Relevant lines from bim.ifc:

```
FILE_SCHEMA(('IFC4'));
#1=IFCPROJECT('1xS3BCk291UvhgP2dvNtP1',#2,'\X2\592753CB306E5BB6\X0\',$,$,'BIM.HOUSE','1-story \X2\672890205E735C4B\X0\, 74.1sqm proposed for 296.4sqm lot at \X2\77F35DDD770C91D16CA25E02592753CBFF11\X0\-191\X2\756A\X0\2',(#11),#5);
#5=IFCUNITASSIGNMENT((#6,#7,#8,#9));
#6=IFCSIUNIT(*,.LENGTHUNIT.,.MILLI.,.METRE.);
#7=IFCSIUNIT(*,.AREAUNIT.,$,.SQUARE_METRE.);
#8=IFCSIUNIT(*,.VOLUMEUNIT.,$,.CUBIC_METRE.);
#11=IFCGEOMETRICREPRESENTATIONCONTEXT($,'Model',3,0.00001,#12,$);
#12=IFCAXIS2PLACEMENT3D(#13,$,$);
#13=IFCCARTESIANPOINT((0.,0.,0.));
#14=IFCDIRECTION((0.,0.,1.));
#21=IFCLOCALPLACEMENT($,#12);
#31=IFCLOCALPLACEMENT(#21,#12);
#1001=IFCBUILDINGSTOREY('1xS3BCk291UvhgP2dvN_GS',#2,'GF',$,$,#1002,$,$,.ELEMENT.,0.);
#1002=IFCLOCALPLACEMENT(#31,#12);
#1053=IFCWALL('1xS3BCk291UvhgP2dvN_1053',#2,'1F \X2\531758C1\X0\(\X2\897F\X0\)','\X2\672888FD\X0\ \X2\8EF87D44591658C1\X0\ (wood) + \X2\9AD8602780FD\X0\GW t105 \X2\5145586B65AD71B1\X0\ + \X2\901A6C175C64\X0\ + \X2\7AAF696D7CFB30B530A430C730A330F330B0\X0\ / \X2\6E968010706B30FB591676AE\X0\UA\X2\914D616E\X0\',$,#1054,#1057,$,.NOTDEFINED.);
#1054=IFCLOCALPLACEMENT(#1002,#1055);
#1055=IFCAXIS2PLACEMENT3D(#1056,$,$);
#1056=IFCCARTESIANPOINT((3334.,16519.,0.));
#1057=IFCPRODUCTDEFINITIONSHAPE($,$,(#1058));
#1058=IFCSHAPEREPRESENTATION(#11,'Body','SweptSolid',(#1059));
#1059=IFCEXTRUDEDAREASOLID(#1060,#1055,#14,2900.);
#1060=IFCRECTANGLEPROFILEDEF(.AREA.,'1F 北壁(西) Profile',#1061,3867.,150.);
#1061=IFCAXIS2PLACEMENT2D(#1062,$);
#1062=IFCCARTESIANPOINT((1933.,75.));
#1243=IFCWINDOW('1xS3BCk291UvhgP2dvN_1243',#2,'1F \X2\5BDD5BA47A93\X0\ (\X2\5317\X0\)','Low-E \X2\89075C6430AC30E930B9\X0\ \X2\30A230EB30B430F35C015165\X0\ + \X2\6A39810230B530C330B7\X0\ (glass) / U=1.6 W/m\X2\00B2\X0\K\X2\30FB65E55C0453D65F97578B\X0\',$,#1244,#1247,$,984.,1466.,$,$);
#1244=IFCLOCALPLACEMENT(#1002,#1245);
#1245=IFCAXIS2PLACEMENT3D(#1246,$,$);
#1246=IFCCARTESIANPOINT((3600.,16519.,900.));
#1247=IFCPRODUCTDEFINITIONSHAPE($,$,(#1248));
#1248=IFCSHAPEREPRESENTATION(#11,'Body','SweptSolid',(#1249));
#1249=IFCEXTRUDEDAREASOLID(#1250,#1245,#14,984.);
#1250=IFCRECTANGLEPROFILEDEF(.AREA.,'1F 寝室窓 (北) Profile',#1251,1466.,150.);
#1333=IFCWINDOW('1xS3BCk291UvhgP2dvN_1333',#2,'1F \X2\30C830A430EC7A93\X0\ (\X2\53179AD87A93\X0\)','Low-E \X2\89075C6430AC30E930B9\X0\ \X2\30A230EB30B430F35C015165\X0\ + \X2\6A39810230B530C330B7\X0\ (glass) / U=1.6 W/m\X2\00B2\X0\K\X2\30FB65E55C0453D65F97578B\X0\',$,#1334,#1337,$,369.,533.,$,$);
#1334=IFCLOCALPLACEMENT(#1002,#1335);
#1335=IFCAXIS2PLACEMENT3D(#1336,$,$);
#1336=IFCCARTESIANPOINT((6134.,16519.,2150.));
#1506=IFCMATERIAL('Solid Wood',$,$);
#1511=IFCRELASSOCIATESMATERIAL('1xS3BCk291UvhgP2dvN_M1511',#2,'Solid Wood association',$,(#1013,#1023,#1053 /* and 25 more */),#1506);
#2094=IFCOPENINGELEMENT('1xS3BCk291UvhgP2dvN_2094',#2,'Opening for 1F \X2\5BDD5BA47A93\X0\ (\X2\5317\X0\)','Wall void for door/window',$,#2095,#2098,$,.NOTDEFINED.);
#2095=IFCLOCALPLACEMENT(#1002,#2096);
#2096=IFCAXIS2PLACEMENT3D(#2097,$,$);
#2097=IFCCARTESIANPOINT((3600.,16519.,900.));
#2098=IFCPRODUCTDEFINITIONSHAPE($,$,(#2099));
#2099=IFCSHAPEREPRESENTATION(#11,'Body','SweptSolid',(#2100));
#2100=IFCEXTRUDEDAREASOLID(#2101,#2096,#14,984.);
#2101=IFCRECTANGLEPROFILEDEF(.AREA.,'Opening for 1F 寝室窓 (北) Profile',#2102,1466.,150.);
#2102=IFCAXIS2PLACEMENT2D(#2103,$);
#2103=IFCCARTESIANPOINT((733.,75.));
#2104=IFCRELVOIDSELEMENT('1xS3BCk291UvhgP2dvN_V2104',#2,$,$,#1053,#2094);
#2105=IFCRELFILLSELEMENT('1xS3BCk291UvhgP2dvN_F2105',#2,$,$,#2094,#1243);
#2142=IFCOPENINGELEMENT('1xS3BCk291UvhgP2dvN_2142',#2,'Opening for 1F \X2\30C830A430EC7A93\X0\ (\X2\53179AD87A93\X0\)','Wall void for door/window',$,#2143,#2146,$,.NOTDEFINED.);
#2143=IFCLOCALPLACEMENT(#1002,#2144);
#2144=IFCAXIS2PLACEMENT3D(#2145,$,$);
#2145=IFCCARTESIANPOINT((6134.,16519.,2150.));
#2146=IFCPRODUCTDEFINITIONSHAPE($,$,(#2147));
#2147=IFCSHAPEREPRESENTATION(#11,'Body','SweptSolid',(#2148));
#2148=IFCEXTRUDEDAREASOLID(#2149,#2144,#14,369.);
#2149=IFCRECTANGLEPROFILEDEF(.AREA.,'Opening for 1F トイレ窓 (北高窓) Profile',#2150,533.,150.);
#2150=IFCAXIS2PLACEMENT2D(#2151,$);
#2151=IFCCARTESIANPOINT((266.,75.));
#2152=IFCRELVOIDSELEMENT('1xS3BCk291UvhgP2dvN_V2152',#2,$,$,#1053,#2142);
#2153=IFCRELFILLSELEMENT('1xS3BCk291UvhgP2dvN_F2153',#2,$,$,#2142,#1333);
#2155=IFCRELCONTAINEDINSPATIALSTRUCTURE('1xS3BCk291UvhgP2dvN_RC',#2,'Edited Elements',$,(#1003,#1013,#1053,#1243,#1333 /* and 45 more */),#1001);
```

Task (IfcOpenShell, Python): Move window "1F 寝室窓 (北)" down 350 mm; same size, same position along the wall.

```python
import numpy as np
import ifcopenshell
import ifcopenshell.api.geometry
import ifcopenshell.util.placement
import ifcopenshell.util.unit

model = ifcopenshell.open("bim.ifc")
unit_scale = ifcopenshell.util.unit.calculate_unit_scale(model)

window = model.by_id(1243)
opening = window.FillsVoids[0].RelatingOpeningElement
dz = -350.0

shift = np.array([0.0, 0.0, dz])
# The window is not placed relative to its opening, so move both.
for product in (opening, window):
    matrix = ifcopenshell.util.placement.get_local_placement(product.ObjectPlacement)
    matrix[:3, 3] += shift
    ifcopenshell.api.geometry.edit_object_placement(model, product=product, matrix=matrix, is_si=False)

print(f"moved by {dz * unit_scale:+.3f} m")

model.write("bim_v2.ifc")
```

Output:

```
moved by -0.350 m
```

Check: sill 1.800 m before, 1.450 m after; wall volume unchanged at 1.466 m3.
